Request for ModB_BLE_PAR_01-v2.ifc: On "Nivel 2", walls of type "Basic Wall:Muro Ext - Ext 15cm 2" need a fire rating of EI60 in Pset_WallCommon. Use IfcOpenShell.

First a look at what the model holds.

```python
import ifcopenshell
import ifcopenshell.util.element

model = ifcopenshell.open("ModB_BLE_PAR_01-v2.ifc")
print(model.schema)
storey = next(s for s in model.by_type("IfcBuildingStorey") if s.Name == "Nivel 2")
walls = [e for e in ifcopenshell.util.element.get_decomposition(storey) if e.is_a("IfcWall")]
seen = {}
for e in walls:
    element_type = ifcopenshell.util.element.get_type(e)
    key = (element_type.Name if element_type != e and element_type else None, ifcopenshell.util.element.get_pset(e, "Pset_WallCommon", "FireRating"))
    seen[key] = seen.get(key, 0) + 1
for (name, value), count in sorted(seen.items(), key=str):
    print(count, "x", name, "|", value)
```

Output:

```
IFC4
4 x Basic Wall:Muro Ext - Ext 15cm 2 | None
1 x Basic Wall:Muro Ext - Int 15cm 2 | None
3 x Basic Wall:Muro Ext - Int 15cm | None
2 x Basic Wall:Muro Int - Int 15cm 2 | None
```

```python
import ifcopenshell
import ifcopenshell.api.pset
import ifcopenshell.util.element

model = ifcopenshell.open("ModB_BLE_PAR_01-v2.ifc")

storey = next(s for s in model.by_type("IfcBuildingStorey") if s.Name == "Nivel 2")
walls = [e for e in ifcopenshell.util.element.get_decomposition(storey) if e.is_a("IfcWall")]

count = 0
for e in walls:
    element_type = ifcopenshell.util.element.get_type(e)
    if element_type in (None, e) or element_type.Name != "Basic Wall:Muro Ext - Ext 15cm 2":
        continue
    # add_pset returns the element's existing set when there is one.
    pset = ifcopenshell.api.pset.add_pset(model, product=e, name="Pset_WallCommon")
    ifcopenshell.api.pset.edit_pset(model, pset=pset, properties={"FireRating": "EI60"})
    count += 1

print(count, "walls updated")

model.write("ModB_BLE_PAR_01-v2_v2.ifc")
```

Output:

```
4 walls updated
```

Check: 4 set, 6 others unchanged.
